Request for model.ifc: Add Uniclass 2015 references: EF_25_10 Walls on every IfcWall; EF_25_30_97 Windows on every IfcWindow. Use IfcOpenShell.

First a look at what the model holds.

```python
import ifcopenshell

model = ifcopenshell.open("model.ifc")
print(model.schema)
print("classifications:", [c.Name for c in model.by_type("IfcClassification")])
for ifc_class in ("IfcDoor", "IfcRoof", "IfcStair", "IfcWall", "IfcWindow"):
    print(ifc_class, len(model.by_type(ifc_class)))
```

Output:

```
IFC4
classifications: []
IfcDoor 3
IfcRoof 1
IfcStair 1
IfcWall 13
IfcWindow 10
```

```python
import ifcopenshell
import ifcopenshell.api.classification

model = ifcopenshell.open("model.ifc")

system = ifcopenshell.api.classification.add_classification(model, classification="Uniclass 2015")

codes = {
    "IfcWall": ("EF_25_10", "Walls"),
    "IfcWindow": ("EF_25_30_97", "Windows"),
}
for ifc_class, (code, name) in codes.items():
    products = model.by_type(ifc_class)
    ifcopenshell.api.classification.add_reference(
        model, products=products, classification=system, identification=code, name=name
    )
    print(code, len(products))

model.write("model-out.ifc")
```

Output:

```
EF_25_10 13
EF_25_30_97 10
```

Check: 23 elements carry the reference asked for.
